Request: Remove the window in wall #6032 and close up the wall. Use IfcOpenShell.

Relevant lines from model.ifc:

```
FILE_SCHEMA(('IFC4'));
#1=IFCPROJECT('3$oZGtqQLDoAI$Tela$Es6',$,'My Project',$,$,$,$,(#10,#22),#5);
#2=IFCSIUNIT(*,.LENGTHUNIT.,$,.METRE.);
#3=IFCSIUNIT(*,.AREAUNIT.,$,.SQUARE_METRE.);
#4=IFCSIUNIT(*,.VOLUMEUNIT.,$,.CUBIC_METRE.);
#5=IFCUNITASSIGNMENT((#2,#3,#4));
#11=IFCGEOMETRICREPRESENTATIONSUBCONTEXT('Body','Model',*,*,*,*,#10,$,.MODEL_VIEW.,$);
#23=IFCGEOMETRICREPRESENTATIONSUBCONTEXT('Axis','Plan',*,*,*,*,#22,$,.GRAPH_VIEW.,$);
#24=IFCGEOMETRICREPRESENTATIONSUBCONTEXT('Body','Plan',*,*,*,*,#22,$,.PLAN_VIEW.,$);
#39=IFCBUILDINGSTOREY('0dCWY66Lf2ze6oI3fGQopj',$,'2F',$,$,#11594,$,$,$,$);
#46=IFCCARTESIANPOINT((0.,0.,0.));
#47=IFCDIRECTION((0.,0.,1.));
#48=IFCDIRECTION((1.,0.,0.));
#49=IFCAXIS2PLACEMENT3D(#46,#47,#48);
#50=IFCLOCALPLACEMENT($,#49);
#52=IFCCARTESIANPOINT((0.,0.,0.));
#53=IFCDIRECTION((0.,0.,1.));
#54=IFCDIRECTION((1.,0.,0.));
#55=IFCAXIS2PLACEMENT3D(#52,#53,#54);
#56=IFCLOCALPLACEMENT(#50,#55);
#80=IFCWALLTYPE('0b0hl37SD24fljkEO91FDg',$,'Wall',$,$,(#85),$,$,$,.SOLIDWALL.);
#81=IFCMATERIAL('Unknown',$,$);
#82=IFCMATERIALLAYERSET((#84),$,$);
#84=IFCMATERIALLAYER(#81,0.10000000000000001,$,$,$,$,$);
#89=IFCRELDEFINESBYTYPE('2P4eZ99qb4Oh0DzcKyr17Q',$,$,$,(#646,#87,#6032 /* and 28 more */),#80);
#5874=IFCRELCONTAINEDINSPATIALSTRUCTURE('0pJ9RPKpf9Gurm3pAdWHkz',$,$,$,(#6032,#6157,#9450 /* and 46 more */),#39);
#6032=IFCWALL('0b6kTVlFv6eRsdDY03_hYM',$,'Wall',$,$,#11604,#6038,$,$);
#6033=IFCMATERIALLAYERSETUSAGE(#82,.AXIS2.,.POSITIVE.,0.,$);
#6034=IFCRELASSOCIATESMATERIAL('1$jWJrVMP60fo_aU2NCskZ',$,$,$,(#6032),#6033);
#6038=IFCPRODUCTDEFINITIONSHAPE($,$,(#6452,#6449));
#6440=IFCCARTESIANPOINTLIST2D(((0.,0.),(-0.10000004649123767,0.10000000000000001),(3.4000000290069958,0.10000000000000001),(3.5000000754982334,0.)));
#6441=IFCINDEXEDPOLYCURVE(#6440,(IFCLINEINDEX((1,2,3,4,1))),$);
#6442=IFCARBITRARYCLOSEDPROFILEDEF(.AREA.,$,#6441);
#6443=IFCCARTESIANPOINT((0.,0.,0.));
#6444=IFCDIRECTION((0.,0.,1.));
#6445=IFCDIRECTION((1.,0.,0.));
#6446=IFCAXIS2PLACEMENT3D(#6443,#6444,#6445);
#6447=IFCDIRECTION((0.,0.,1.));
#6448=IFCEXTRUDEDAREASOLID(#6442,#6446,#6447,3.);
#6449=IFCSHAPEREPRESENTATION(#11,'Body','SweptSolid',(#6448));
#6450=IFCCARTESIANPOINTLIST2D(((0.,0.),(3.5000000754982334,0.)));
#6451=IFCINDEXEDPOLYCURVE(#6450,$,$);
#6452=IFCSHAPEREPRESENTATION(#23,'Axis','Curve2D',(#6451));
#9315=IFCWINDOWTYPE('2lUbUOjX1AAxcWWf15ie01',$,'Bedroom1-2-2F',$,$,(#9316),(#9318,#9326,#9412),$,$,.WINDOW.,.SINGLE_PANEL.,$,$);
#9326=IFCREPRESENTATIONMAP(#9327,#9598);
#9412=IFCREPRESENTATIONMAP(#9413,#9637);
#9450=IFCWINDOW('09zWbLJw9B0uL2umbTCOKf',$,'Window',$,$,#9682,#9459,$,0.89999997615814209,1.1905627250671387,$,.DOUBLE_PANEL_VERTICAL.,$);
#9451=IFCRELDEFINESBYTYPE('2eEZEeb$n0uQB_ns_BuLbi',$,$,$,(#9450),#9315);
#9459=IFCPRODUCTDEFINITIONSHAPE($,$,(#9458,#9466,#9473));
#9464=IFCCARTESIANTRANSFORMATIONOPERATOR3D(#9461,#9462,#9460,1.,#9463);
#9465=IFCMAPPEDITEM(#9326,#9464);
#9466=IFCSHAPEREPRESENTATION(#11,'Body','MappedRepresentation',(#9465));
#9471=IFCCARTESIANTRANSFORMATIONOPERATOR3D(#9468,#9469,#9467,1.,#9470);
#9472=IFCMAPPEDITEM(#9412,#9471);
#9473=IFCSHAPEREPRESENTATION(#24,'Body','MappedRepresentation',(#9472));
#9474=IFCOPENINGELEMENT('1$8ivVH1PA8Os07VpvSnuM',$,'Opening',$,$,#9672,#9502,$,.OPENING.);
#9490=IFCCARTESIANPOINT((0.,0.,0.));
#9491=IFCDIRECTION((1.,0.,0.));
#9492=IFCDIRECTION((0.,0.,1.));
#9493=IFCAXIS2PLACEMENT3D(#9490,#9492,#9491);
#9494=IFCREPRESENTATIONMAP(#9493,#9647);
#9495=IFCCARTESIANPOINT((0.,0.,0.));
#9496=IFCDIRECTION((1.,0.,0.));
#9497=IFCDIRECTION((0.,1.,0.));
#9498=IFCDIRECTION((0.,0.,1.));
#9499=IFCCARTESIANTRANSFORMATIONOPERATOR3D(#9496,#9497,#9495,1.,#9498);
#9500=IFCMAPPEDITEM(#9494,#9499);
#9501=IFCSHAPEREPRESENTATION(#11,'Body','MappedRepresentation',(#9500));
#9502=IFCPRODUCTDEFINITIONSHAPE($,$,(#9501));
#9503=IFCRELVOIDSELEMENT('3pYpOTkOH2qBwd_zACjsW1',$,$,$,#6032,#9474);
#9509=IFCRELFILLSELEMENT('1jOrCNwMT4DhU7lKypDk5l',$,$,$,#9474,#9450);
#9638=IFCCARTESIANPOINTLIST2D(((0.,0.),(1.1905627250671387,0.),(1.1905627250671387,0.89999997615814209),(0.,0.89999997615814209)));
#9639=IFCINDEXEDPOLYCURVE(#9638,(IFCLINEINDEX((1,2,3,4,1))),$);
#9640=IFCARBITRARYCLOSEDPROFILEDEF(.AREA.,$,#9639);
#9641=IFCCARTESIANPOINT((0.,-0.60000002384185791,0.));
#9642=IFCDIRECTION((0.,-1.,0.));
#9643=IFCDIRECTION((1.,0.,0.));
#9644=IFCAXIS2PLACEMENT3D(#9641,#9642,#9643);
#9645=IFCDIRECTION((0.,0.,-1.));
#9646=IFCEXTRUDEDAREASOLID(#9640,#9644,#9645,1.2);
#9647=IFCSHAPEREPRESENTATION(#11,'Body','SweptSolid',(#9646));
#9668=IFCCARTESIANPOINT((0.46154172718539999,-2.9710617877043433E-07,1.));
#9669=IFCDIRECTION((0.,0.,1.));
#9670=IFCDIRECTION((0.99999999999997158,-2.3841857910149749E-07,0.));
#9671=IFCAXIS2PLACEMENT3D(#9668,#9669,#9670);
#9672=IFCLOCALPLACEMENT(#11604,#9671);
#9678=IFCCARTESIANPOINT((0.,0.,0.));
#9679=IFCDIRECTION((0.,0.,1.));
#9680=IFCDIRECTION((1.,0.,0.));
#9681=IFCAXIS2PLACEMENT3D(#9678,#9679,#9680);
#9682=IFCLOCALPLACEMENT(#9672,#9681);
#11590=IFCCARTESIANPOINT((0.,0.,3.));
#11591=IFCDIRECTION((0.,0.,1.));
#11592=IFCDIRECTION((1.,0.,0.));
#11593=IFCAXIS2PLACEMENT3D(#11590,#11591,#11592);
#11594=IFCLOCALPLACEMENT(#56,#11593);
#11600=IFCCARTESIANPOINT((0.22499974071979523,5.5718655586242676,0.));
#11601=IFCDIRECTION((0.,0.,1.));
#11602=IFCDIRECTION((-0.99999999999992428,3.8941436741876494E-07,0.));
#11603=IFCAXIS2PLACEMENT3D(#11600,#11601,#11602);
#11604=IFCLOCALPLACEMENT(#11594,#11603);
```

```python
import ifcopenshell
import ifcopenshell.api.feature
import ifcopenshell.api.root
import ifcopenshell.geom
import ifcopenshell.util.shape

model = ifcopenshell.open("model.ifc")
settings = ifcopenshell.geom.settings()


def volume(element):
    """Net volume in cubic metres, openings subtracted."""
    shape = ifcopenshell.geom.create_shape(settings, element)
    return ifcopenshell.util.shape.get_volume(shape.geometry)


window = model.by_guid("09zWbLJw9B0uL2umbTCOKf")
opening = window.FillsVoids[0].RelatingOpeningElement
wall = opening.VoidsElements[0].RelatingBuildingElement
before = volume(wall)

ifcopenshell.api.root.remove_product(model, product=window)
ifcopenshell.api.feature.remove_feature(model, feature=opening)

after = volume(wall)

print(f"wall volume {before:.3f} -> {after:.3f} m3")

model.write("model_rev.ifc")
```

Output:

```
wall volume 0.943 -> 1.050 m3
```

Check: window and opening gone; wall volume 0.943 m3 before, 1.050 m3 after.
